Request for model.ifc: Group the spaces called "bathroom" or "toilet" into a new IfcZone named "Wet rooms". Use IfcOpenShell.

First a look at what the model holds.

```python
import ifcopenshell

model = ifcopenshell.open("model.ifc")
print(model.schema)
seen = {}
for space in model.by_type("IfcSpace"):
    seen[space.LongName] = seen.get(space.LongName, 0) + 1
for name, count in sorted(seen.items(), key=str):
    print(count, "x", name)
print("zones:", [z.Name for z in model.by_type("IfcZone")][:20])
```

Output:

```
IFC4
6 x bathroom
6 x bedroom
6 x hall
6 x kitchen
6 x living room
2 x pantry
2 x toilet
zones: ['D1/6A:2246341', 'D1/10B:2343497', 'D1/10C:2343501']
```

```python
import ifcopenshell
import ifcopenshell.api.group
import ifcopenshell.api.root

model = ifcopenshell.open("model.ifc")

names = {"bathroom", "toilet"}
spaces = [s for s in model.by_type("IfcSpace") if s.LongName in names]

zone = ifcopenshell.api.root.create_entity(model, ifc_class="IfcZone", name="Wet rooms")
ifcopenshell.api.group.assign_group(model, products=spaces, group=zone)
print(len(spaces), "spaces in", zone.Name)

model.write("model_edited.ifc")
```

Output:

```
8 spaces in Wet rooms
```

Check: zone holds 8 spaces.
